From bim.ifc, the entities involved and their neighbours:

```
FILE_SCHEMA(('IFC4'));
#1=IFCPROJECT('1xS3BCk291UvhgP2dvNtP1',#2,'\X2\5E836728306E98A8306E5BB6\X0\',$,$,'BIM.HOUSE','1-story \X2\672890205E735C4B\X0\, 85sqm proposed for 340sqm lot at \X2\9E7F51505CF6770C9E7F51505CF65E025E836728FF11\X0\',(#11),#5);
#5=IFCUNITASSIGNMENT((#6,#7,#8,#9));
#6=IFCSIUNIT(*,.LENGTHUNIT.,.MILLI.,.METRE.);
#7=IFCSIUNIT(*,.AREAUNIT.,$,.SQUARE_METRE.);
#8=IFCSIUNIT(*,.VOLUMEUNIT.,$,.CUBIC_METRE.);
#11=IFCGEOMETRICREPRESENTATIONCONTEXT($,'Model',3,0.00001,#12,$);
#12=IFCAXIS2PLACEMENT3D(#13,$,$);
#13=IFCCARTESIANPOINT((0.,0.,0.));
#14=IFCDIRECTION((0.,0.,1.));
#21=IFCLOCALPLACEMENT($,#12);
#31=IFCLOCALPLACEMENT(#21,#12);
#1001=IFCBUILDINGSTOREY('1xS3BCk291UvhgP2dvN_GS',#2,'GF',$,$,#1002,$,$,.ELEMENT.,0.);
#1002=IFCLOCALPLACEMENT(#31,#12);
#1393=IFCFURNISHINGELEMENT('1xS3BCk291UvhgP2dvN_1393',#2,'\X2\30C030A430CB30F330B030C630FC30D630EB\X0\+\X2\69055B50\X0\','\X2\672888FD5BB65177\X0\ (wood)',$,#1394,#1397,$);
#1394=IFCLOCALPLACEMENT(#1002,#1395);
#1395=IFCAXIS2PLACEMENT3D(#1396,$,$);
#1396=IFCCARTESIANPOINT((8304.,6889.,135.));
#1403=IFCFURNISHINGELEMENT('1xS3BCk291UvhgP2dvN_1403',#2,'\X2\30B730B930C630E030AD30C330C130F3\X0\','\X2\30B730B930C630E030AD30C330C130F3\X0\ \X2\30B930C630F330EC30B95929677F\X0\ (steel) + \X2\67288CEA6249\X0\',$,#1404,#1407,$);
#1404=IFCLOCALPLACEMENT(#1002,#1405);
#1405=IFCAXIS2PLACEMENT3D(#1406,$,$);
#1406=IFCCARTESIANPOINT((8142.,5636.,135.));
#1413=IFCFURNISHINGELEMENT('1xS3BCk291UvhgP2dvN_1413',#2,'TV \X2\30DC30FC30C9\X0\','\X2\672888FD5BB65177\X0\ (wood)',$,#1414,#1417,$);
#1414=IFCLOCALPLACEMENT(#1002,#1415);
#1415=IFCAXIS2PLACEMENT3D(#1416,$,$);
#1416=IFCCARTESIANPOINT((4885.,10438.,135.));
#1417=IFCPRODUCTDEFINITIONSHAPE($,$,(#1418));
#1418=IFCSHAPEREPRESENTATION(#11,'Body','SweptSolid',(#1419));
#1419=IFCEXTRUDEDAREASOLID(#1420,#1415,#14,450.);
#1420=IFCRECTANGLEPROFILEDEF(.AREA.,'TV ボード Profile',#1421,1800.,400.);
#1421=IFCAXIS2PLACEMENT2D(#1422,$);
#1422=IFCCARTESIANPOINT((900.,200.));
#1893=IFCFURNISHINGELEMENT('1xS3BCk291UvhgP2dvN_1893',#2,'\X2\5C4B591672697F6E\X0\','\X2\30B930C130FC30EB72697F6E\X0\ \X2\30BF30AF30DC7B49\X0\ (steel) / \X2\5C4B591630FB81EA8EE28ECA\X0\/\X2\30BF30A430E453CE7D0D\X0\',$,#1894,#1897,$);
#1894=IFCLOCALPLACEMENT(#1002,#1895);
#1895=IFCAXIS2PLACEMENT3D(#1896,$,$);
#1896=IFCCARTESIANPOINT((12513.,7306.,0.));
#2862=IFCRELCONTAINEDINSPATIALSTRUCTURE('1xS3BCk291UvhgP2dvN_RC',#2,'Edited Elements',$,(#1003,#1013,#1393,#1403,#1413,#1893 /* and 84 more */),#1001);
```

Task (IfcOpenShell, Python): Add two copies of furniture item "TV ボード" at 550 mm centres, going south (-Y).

```python
import numpy as np
import ifcopenshell
import ifcopenshell.api.geometry
import ifcopenshell.api.root
import ifcopenshell.util.element
import ifcopenshell.util.placement

model = ifcopenshell.open("bim.ifc")


def reuse_history(source, copy):
    """copy_class also copies each property set's owner history, people and application; keep the originals."""
    for rel in copy.IsDefinedBy:
        if rel.is_a("IfcRelDefinesByProperties") and (history := rel.RelatingPropertyDefinition.OwnerHistory):
            rel.RelatingPropertyDefinition.OwnerHistory = source.OwnerHistory
            ifcopenshell.util.element.remove_deep2(model, history)


source = model.by_guid("1xS3BCk291UvhgP2dvN_1413")
base = ifcopenshell.util.placement.get_local_placement(source.ObjectPlacement)
step = np.array([0.0, -1.0, 0.0]) * 550.0

for i in range(1, 3):
    copy = ifcopenshell.api.root.copy_class(model, product=source)
    copy.Representation = ifcopenshell.util.element.copy_deep(
        model, source.Representation, exclude=["IfcGeometricRepresentationContext", "IfcRepresentationMap"]
    )
    reuse_history(source, copy)
    matrix = base.copy()
    matrix[:3, 3] += i * step
    print("added at", matrix[:3, 3].round(3) + 0.0)
    ifcopenshell.api.geometry.edit_object_placement(model, product=copy, matrix=matrix, is_si=False)

model.write("bim_v2.ifc")
```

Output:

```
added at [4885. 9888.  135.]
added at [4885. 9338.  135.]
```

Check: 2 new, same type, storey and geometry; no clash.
